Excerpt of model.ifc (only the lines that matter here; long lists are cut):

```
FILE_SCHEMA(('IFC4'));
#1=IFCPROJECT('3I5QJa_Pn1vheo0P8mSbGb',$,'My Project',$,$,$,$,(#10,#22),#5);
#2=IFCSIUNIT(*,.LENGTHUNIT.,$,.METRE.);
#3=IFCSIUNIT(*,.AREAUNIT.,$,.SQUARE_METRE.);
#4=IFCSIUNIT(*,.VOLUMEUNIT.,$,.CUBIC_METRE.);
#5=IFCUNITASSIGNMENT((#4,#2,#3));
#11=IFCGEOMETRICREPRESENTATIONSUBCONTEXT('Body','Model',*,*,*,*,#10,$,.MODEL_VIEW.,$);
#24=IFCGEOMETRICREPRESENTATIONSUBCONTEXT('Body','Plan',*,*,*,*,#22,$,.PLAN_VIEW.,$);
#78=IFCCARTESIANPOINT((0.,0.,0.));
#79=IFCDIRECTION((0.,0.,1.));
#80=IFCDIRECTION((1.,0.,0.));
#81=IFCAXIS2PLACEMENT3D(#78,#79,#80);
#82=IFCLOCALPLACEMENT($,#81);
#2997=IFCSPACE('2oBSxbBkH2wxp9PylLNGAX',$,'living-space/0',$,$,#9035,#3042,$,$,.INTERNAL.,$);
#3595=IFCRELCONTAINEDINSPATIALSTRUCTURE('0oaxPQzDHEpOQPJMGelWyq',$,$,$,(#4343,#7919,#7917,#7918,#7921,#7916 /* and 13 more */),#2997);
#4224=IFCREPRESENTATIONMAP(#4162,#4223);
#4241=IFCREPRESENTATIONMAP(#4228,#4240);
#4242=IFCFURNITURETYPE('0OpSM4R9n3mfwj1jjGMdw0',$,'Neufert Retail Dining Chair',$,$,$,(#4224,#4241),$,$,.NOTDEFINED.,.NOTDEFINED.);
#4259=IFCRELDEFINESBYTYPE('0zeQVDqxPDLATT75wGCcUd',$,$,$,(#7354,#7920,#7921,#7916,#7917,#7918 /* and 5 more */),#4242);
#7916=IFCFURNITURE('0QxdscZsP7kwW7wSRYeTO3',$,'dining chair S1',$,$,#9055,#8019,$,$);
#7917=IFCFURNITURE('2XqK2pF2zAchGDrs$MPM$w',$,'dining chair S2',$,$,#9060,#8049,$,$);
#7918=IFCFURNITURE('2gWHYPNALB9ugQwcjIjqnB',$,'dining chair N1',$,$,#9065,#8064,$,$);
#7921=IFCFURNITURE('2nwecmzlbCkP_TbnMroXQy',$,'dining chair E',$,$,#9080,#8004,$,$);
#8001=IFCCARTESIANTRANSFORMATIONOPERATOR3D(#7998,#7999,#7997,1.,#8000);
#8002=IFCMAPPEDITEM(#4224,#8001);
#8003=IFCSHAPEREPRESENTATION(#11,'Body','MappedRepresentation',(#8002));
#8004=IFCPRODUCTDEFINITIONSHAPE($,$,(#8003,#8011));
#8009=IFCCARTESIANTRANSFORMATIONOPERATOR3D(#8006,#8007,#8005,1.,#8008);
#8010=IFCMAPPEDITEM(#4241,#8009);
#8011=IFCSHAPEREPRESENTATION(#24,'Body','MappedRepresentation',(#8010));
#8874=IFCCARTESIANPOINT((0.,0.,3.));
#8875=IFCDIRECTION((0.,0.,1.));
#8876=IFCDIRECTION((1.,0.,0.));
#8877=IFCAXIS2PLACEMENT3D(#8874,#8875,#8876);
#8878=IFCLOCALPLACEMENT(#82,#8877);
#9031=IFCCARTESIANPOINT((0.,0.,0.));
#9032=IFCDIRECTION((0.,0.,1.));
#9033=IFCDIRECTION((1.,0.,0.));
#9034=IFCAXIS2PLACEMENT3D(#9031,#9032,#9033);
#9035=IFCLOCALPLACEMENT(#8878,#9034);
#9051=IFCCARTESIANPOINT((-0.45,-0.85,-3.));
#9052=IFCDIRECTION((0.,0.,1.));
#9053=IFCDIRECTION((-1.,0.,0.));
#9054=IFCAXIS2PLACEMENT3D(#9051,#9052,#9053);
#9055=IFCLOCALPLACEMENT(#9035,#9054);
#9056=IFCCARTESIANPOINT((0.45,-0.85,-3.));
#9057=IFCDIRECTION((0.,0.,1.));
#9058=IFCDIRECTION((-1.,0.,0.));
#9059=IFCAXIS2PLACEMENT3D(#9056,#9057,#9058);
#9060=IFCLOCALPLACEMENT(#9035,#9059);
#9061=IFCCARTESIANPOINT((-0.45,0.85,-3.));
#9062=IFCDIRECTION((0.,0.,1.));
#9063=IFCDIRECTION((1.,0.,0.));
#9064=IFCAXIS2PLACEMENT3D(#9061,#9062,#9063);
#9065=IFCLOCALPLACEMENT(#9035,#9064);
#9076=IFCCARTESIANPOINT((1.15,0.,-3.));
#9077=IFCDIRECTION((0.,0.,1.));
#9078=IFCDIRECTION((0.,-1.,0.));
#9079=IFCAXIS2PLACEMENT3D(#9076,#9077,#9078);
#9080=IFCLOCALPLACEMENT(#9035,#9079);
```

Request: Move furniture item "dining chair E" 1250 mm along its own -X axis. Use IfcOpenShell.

```python
import ifcopenshell
import ifcopenshell.api.geometry
import ifcopenshell.util.placement

model = ifcopenshell.open("model.ifc")

item = model.by_guid("2nwecmzlbCkP_TbnMroXQy")
matrix = ifcopenshell.util.placement.get_local_placement(item.ObjectPlacement)
matrix[:3, 3] -= matrix[:3, 0] * 1.25
ifcopenshell.api.geometry.edit_object_placement(model, product=item, matrix=matrix, is_si=False)

print(ifcopenshell.util.placement.get_local_placement(item.ObjectPlacement).round(3) + 0.0)

model.write("model_edited.ifc")
```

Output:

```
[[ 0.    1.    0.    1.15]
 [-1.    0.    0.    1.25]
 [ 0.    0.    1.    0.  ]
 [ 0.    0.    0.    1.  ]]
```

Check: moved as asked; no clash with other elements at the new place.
